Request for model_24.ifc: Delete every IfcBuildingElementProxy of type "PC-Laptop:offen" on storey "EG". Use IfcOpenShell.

First a look at what the model holds.

```python
import ifcopenshell
import ifcopenshell.util.element

model = ifcopenshell.open("model_24.ifc")
print(model.schema)
storey = next(s for s in model.by_type("IfcBuildingStorey") if s.Name == "EG")
proxies = [e for e in ifcopenshell.util.element.get_decomposition(storey) if e.is_a("IfcBuildingElementProxy")]
seen = {}
for e in proxies:
    element_type = ifcopenshell.util.element.get_type(e)
    name = element_type.Name if element_type not in (None, e) else None
    seen[name] = seen.get(name, 0) + 1
for name, count in sorted(seen.items(), key=str):
    print(count, "x", name)
```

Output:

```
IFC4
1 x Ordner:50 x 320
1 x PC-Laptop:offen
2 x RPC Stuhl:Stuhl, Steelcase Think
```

```python
import ifcopenshell
import ifcopenshell.api.root
import ifcopenshell.util.element

model = ifcopenshell.open("model_24.ifc")

storey = next(s for s in model.by_type("IfcBuildingStorey") if s.Name == "EG")
proxies = [e for e in ifcopenshell.util.element.get_decomposition(storey) if e.is_a("IfcBuildingElementProxy")]
targets = [e for e in proxies if (t := ifcopenshell.util.element.get_type(e)) not in (None, e) and t.Name == "PC-Laptop:offen"]

for e in targets:
    ifcopenshell.api.root.remove_product(model, product=e)
print(len(targets), "removed")

model.write("model_24-out.ifc")
```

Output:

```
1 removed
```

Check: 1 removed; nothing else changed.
